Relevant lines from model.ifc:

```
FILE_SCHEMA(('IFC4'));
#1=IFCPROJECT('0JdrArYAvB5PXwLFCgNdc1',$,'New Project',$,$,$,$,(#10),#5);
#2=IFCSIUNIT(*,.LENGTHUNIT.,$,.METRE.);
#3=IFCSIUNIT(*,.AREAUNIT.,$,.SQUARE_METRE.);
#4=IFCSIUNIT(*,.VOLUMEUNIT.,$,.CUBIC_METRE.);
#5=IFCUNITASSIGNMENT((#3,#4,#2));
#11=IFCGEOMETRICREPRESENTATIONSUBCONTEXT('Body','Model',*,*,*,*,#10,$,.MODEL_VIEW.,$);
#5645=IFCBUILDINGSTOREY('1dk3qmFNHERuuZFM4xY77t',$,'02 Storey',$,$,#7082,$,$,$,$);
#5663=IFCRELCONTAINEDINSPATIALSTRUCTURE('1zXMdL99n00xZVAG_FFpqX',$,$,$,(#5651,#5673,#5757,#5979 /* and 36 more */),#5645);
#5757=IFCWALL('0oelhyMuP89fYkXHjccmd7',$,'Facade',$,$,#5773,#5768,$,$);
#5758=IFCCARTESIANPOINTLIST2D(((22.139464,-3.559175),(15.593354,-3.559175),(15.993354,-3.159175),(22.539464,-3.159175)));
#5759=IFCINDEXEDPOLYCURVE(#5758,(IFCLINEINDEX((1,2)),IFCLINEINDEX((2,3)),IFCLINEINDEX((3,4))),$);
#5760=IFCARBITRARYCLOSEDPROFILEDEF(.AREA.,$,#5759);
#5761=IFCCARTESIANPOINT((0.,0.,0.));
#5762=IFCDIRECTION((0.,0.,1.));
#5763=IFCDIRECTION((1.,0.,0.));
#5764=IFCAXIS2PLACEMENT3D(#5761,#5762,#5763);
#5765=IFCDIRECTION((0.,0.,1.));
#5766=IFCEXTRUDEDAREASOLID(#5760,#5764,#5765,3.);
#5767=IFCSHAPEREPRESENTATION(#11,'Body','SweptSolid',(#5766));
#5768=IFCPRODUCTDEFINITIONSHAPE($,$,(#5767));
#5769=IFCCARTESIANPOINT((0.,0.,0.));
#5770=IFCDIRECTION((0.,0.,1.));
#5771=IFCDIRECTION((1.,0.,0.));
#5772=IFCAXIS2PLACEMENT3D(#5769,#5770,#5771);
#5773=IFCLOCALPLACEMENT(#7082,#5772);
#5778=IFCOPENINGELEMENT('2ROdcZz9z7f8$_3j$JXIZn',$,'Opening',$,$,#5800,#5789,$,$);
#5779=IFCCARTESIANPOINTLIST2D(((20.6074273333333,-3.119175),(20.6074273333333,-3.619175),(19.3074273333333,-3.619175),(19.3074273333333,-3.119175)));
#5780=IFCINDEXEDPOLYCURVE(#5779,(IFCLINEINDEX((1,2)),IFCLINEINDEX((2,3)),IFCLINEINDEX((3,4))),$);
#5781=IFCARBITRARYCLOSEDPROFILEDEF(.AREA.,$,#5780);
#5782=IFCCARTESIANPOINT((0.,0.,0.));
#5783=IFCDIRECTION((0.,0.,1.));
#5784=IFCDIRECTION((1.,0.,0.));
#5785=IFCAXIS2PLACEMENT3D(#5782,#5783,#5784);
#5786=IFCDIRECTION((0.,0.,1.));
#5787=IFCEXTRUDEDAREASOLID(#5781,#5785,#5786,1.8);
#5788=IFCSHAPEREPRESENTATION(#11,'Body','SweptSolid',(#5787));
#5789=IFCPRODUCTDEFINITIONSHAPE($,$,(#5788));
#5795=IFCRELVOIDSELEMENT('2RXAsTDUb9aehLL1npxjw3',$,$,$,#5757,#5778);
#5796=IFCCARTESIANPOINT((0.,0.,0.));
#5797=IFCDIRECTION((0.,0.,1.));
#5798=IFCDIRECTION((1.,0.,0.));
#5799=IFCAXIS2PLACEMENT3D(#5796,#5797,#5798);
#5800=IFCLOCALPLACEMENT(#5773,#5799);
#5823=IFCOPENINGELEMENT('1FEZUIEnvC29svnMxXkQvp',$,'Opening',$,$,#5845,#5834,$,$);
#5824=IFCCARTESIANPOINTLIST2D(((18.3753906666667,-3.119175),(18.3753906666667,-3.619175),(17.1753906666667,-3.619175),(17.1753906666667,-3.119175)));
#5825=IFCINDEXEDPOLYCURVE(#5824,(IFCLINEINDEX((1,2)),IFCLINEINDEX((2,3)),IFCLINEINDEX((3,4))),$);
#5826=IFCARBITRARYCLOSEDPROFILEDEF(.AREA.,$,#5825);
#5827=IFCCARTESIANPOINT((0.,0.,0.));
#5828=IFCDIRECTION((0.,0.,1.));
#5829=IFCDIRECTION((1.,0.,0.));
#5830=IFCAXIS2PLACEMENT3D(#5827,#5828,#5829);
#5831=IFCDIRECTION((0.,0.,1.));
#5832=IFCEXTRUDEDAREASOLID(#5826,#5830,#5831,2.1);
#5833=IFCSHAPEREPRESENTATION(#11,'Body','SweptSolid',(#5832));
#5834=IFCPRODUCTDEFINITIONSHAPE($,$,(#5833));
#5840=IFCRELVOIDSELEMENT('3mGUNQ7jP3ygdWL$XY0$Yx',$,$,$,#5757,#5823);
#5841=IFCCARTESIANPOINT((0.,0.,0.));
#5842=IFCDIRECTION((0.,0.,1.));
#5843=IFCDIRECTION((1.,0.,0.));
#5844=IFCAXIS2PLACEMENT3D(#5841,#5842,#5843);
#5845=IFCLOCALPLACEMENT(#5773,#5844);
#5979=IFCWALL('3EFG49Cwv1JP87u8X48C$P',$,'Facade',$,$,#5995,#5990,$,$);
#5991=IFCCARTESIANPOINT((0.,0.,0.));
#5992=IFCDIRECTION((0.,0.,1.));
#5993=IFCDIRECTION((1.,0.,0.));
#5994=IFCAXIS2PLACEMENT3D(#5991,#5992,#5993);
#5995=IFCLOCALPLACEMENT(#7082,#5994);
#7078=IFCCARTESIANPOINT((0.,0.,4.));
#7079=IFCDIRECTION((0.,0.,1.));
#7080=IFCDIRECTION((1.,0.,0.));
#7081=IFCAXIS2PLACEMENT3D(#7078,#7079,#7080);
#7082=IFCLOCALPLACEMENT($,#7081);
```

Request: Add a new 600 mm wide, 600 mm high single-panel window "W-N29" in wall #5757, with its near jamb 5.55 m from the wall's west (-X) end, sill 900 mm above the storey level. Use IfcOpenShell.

```python
import numpy as np
import ifcopenshell
import ifcopenshell.api.feature
import ifcopenshell.api.geometry
import ifcopenshell.api.root
import ifcopenshell.api.spatial
import ifcopenshell.geom
import ifcopenshell.util.element
import ifcopenshell.util.placement
import ifcopenshell.util.representation
import ifcopenshell.util.shape
import ifcopenshell.util.unit

model = ifcopenshell.open("model.ifc")
unit_scale = ifcopenshell.util.unit.calculate_unit_scale(model)
settings = ifcopenshell.geom.settings()


def volume(element):
    """Net volume in cubic metres, openings subtracted."""
    shape = ifcopenshell.geom.create_shape(settings, element)
    return ifcopenshell.util.shape.get_volume(shape.geometry)


wall = model.by_id(5757)
storey = ifcopenshell.util.element.get_container(wall, ifc_class="IfcBuildingStorey")
context = ifcopenshell.util.representation.get_context(model, "Model", "Body", "MODEL_VIEW")
before = volume(wall)

width, height, from_end, sill = 0.6, 0.6, 5.55, 0.9  # metres

# The wall runs along its own X axis, and the end named is its -X end.
wall_shape = ifcopenshell.geom.create_shape(settings, wall)
x, y, z = ifcopenshell.util.shape.get_vertices(wall_shape.geometry).T
start = x.min() + from_end
face, thickness = float(y.min()), float(y.max() - y.min())
wall_matrix = ifcopenshell.util.placement.get_local_placement(wall.ObjectPlacement)
level = ifcopenshell.util.placement.get_local_placement(storey.ObjectPlacement)[2, 3]


def in_wall(x, y):
    """Placement at x, y metres in the wall's axes, at sill height."""
    matrix = wall_matrix.copy()
    matrix[:, 3] = wall_matrix @ np.array([x / unit_scale, y / unit_scale, 0.0, 1.0])
    matrix[2, 3] = level + sill / unit_scale
    return matrix


# Opening: a box that overshoots both wall faces by 50 mm.
opening = ifcopenshell.api.root.create_entity(model, ifc_class="IfcOpeningElement", predefined_type="OPENING")
box = ifcopenshell.api.geometry.add_wall_representation(
    model, context=context, length=width, height=height, thickness=thickness + 0.1
)
ifcopenshell.api.geometry.assign_representation(model, product=opening, representation=box)
ifcopenshell.api.geometry.edit_object_placement(model, product=opening, matrix=in_wall(start, face - 0.05), is_si=False)
ifcopenshell.api.feature.add_feature(model, feature=opening, element=wall)

window = ifcopenshell.api.root.create_entity(model, ifc_class="IfcWindow", name="W-N29", predefined_type="WINDOW")
window.OverallWidth, window.OverallHeight = width / unit_scale, height / unit_scale
window.PartitioningType = "SINGLE_PANEL"
body = ifcopenshell.api.geometry.add_window_representation(
    model,
    context=context,
    overall_width=window.OverallWidth,
    overall_height=window.OverallHeight,
    partition_type="SINGLE_PANEL",
)
ifcopenshell.api.geometry.assign_representation(model, product=window, representation=body)
ifcopenshell.api.spatial.assign_container(model, products=[window], relating_structure=storey)
ifcopenshell.api.feature.add_filling(model, opening=opening, element=window)

# Centre the window in the wall's thickness.
ifcopenshell.api.geometry.edit_object_placement(model, product=window, matrix=in_wall(start, face), is_si=False)
window_shape = ifcopenshell.geom.create_shape(settings, window)
depth = ifcopenshell.util.shape.get_vertices(window_shape.geometry)[:, 1]
offset = face + thickness / 2 - (depth.min() + depth.max()) / 2
ifcopenshell.api.geometry.edit_object_placement(model, product=window, matrix=in_wall(start, offset), is_si=False)

after = volume(wall)

print(f"wall volume {before:.3f} -> {after:.3f} m3")

model.write("model_edited.ifc")
```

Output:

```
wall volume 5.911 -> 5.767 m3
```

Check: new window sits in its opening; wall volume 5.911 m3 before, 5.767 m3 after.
